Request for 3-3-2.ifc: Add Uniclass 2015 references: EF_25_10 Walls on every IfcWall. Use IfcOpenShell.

First a look at what the model holds.

```python
import ifcopenshell

model = ifcopenshell.open("3-3-2.ifc")
print(model.schema)
print("classifications:", [c.Name for c in model.by_type("IfcClassification")])
for ifc_class in ("IfcDoor", "IfcRoof", "IfcStair", "IfcWall", "IfcWindow"):
    print(ifc_class, len(model.by_type(ifc_class)))
```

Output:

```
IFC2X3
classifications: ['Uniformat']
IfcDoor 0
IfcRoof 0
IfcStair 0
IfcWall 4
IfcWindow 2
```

```python
import ifcopenshell
import ifcopenshell.api.classification

model = ifcopenshell.open("3-3-2.ifc")

# IFC2X3 requires Source and Edition and has no link from the project to the system.
system = model.create_entity("IfcClassification", Source="NBS", Edition="2015", Name="Uniclass 2015")

codes = {
    "IfcWall": ("EF_25_10", "Walls"),
}
for ifc_class, (code, name) in codes.items():
    products = model.by_type(ifc_class)
    ifcopenshell.api.classification.add_reference(
        model, products=products, classification=system, identification=code, name=name
    )
    print(code, len(products))

model.write("3-3-2_v2.ifc")
```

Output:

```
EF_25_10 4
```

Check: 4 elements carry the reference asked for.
